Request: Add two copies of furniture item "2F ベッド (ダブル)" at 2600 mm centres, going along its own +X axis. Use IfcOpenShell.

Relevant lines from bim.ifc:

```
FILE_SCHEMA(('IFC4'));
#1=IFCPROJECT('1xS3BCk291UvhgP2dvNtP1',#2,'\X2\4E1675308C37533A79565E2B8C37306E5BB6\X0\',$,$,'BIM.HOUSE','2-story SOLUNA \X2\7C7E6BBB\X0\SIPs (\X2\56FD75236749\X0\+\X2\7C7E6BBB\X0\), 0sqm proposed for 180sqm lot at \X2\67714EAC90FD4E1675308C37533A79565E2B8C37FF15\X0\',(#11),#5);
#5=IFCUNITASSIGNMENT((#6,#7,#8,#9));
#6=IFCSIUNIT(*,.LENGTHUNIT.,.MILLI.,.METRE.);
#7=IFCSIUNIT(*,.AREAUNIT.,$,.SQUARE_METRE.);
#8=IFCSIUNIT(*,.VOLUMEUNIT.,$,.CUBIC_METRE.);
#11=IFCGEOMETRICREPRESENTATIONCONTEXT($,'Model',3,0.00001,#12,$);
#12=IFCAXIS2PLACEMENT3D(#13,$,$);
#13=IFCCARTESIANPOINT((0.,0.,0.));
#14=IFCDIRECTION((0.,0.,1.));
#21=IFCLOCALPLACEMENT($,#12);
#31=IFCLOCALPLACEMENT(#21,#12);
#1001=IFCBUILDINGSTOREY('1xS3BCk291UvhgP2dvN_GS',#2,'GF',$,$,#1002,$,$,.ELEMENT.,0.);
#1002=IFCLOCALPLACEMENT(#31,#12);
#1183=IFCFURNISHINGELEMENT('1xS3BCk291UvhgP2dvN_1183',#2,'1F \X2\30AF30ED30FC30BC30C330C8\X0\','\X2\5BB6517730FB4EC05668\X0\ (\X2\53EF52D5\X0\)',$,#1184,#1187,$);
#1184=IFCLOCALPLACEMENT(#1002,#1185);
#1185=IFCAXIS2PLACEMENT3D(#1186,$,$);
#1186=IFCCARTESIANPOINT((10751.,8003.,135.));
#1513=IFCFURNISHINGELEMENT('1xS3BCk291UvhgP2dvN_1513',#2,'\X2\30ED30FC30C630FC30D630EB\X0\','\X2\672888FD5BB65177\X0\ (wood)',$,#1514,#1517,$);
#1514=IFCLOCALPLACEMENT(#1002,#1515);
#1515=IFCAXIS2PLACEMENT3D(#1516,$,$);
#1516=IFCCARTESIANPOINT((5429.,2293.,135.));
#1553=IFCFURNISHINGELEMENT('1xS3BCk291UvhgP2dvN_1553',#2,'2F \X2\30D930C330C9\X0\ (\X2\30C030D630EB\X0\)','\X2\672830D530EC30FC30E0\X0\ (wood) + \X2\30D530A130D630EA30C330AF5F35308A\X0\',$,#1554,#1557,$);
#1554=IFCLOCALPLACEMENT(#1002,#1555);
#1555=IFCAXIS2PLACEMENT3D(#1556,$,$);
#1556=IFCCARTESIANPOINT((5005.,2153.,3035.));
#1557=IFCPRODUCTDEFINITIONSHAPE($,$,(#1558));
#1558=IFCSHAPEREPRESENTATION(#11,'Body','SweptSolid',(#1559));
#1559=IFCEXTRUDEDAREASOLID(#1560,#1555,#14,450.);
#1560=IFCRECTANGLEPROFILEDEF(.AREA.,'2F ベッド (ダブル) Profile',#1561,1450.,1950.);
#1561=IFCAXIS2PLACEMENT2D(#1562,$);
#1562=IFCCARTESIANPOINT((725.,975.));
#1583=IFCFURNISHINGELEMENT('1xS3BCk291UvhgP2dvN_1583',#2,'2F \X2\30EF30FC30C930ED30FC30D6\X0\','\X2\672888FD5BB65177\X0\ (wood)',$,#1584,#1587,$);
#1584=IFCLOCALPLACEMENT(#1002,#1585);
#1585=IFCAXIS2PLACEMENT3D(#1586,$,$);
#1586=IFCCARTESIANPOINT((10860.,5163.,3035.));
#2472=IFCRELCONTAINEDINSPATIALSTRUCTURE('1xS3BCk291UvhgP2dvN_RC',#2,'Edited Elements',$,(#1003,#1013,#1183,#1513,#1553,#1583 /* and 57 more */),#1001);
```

```python
import ifcopenshell
import ifcopenshell.api.geometry
import ifcopenshell.api.root
import ifcopenshell.util.element
import ifcopenshell.util.placement
import ifcopenshell.util.unit

model = ifcopenshell.open("bim.ifc")
unit_scale = ifcopenshell.util.unit.calculate_unit_scale(model)


def reuse_history(source, copy):
    """copy_class also copies each property set's owner history, people and application; keep the originals."""
    for rel in copy.IsDefinedBy:
        if rel.is_a("IfcRelDefinesByProperties") and (history := rel.RelatingPropertyDefinition.OwnerHistory):
            rel.RelatingPropertyDefinition.OwnerHistory = source.OwnerHistory
            ifcopenshell.util.element.remove_deep2(model, history)


source = model.by_guid("1xS3BCk291UvhgP2dvN_1553")
base = ifcopenshell.util.placement.get_local_placement(source.ObjectPlacement)
step = base[:3, 0] * 2.6 / unit_scale

for i in range(1, 3):
    copy = ifcopenshell.api.root.copy_class(model, product=source)
    copy.Representation = ifcopenshell.util.element.copy_deep(
        model, source.Representation, exclude=["IfcGeometricRepresentationContext", "IfcRepresentationMap"]
    )
    reuse_history(source, copy)
    matrix = base.copy()
    matrix[:3, 3] += i * step
    print("added at", matrix[:3, 3].round(3) + 0.0)
    ifcopenshell.api.geometry.edit_object_placement(model, product=copy, matrix=matrix, is_si=False)

model.write("bim-out.ifc")
```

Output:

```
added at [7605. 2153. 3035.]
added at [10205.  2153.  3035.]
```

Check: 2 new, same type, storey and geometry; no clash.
